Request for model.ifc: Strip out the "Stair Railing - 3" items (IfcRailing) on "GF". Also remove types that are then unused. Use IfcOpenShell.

First a look at what the model holds.

```python
import ifcopenshell
import ifcopenshell.util.element

model = ifcopenshell.open("model.ifc")
print(model.schema)
storey = next(s for s in model.by_type("IfcBuildingStorey") if s.Name == "GF")
railings = [e for e in ifcopenshell.util.element.get_decomposition(storey) if e.is_a("IfcRailing")]
seen = {}
for e in railings:
    element_type = ifcopenshell.util.element.get_type(e)
    name = element_type.Name if element_type not in (None, e) else None
    seen[name] = seen.get(name, 0) + 1
for name, count in sorted(seen.items(), key=str):
    print(count, "x", name)
```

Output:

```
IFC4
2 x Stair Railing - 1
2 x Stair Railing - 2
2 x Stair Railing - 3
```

```python
import ifcopenshell
import ifcopenshell.api.root
import ifcopenshell.util.element

model = ifcopenshell.open("model.ifc")

storey = next(s for s in model.by_type("IfcBuildingStorey") if s.Name == "GF")
railings = [e for e in ifcopenshell.util.element.get_decomposition(storey) if e.is_a("IfcRailing")]
targets = [e for e in railings if (t := ifcopenshell.util.element.get_type(e)) not in (None, e) and t.Name == "Stair Railing - 3"]
types = {ifcopenshell.util.element.get_type(e) for e in targets} - {None, *targets}

for e in targets:
    ifcopenshell.api.root.remove_product(model, product=e)
print(len(targets), "removed")

unused = [t for t in types if not ifcopenshell.util.element.get_types(t)]
for t in unused:
    ifcopenshell.api.root.remove_product(model, product=t)
print(len(unused), "unused types removed")

model.write("model_v2.ifc")
```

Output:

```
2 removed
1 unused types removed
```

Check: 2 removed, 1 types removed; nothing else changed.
